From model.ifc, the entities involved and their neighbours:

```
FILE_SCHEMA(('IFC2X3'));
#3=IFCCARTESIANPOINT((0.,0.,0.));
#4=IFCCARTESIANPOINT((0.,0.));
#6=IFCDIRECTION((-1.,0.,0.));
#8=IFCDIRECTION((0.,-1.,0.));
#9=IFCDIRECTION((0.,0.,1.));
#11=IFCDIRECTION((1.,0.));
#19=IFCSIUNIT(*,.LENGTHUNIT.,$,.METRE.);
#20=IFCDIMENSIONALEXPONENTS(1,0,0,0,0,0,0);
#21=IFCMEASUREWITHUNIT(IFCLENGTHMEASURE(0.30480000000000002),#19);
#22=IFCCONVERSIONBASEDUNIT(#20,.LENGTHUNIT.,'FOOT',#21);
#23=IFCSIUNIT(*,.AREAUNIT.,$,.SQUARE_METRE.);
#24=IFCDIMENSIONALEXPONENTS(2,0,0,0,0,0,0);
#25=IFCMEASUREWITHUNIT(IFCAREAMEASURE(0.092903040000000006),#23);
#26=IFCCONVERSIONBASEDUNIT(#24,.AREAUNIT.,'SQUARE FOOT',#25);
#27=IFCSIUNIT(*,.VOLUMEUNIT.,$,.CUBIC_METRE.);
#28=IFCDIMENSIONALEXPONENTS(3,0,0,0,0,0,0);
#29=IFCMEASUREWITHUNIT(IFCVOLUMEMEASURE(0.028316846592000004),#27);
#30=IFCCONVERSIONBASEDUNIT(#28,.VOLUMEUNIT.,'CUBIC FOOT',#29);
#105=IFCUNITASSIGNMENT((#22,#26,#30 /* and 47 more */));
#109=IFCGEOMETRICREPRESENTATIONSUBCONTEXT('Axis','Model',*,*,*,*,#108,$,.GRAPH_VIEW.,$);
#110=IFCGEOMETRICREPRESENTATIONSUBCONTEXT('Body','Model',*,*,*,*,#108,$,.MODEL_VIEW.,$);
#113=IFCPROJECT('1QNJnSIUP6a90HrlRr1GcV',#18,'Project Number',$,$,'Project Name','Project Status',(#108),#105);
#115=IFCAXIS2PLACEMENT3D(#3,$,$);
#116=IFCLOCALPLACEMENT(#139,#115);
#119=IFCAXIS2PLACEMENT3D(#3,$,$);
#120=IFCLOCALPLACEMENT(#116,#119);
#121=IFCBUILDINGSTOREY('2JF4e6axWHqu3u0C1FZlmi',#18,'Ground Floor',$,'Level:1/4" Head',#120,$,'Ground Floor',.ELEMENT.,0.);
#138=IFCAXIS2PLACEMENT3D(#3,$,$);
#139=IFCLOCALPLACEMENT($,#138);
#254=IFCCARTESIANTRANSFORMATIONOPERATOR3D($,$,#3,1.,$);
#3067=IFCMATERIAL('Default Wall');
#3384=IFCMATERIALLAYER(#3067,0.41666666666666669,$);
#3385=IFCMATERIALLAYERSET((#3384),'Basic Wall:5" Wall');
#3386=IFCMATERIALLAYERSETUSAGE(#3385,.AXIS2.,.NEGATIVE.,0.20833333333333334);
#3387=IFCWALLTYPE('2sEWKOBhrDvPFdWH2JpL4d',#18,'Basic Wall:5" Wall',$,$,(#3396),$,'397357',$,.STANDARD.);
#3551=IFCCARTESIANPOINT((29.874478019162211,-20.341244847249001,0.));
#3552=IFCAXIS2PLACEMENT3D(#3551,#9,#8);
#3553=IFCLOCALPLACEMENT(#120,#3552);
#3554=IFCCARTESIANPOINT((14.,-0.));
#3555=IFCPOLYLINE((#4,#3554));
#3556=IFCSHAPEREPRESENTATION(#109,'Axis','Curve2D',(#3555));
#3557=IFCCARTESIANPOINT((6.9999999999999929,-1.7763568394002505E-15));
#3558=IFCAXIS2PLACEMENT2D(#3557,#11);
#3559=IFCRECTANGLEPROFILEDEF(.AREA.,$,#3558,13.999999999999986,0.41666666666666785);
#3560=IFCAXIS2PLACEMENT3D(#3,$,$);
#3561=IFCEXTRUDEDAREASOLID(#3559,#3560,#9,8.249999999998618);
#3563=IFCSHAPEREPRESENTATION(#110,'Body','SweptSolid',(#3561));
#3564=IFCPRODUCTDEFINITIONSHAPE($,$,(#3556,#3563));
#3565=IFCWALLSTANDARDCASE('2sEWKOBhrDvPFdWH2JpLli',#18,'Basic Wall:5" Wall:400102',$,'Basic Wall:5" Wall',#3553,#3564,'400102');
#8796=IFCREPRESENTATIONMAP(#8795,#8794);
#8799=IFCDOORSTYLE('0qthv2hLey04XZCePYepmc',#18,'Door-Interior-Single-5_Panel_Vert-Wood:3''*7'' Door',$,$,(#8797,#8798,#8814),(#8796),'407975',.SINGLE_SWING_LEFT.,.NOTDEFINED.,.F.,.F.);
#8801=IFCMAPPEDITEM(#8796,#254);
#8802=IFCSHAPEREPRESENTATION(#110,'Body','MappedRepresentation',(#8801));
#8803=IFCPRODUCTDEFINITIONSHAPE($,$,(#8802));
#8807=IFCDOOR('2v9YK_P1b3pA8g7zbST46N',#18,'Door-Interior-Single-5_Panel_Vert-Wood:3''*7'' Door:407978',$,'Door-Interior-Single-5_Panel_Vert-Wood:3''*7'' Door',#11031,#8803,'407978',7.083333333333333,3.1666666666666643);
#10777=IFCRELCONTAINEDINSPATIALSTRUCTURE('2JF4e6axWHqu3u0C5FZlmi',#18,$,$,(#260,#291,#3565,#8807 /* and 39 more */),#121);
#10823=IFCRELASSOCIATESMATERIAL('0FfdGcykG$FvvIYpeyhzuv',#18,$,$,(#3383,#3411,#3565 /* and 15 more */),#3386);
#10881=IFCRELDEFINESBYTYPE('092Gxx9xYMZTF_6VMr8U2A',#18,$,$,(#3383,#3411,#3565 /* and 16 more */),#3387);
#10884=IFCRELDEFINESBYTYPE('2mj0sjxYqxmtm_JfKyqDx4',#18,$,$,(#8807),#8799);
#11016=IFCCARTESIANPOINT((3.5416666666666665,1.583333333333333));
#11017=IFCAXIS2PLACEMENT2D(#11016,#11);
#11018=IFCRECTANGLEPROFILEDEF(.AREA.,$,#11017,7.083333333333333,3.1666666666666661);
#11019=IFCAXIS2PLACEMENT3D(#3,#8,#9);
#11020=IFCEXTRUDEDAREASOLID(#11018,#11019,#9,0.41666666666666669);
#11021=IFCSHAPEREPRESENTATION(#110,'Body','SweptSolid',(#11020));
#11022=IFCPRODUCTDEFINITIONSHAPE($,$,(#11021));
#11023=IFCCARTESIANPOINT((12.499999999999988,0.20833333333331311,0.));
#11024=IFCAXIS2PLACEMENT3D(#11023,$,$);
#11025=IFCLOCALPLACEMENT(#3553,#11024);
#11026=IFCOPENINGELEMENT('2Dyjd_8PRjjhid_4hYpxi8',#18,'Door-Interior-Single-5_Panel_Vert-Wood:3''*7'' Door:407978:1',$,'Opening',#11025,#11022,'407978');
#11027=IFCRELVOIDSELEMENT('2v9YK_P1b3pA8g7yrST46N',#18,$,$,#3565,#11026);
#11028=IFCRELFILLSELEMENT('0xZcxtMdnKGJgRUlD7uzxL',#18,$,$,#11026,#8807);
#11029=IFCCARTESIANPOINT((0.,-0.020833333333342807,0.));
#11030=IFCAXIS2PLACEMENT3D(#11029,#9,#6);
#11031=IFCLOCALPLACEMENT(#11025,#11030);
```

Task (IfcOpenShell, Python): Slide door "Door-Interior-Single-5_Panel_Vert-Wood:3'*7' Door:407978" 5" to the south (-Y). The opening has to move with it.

```python
import ifcopenshell
import ifcopenshell.api.geometry
import ifcopenshell.util.placement
import ifcopenshell.util.unit

model = ifcopenshell.open("model.ifc")
unit_scale = ifcopenshell.util.unit.calculate_unit_scale(model)

door = model.by_guid("2v9YK_P1b3pA8g7zbST46N")
opening = door.FillsVoids[0].RelatingOpeningElement
wall = opening.VoidsElements[0].RelatingBuildingElement

wall_matrix = ifcopenshell.util.placement.get_local_placement(wall.ObjectPlacement)
shift = wall_matrix[:3, 0] * 5 * 0.0254 / unit_scale
before = ifcopenshell.util.placement.get_local_placement(door.ObjectPlacement)[:3, 3].copy()

# The door is placed relative to its opening, so it follows when the opening moves.
matrix = ifcopenshell.util.placement.get_local_placement(opening.ObjectPlacement)
matrix[:3, 3] += shift
ifcopenshell.api.geometry.edit_object_placement(
    model, product=opening, matrix=matrix, is_si=False, should_transform_children=True
)

after = ifcopenshell.util.placement.get_local_placement(door.ObjectPlacement)[:3, 3]
print("door moved by", (after - before).round(3) + 0.0)

model.write("model_edited.ifc")
```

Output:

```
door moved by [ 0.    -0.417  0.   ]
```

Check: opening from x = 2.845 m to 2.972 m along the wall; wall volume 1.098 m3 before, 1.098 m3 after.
